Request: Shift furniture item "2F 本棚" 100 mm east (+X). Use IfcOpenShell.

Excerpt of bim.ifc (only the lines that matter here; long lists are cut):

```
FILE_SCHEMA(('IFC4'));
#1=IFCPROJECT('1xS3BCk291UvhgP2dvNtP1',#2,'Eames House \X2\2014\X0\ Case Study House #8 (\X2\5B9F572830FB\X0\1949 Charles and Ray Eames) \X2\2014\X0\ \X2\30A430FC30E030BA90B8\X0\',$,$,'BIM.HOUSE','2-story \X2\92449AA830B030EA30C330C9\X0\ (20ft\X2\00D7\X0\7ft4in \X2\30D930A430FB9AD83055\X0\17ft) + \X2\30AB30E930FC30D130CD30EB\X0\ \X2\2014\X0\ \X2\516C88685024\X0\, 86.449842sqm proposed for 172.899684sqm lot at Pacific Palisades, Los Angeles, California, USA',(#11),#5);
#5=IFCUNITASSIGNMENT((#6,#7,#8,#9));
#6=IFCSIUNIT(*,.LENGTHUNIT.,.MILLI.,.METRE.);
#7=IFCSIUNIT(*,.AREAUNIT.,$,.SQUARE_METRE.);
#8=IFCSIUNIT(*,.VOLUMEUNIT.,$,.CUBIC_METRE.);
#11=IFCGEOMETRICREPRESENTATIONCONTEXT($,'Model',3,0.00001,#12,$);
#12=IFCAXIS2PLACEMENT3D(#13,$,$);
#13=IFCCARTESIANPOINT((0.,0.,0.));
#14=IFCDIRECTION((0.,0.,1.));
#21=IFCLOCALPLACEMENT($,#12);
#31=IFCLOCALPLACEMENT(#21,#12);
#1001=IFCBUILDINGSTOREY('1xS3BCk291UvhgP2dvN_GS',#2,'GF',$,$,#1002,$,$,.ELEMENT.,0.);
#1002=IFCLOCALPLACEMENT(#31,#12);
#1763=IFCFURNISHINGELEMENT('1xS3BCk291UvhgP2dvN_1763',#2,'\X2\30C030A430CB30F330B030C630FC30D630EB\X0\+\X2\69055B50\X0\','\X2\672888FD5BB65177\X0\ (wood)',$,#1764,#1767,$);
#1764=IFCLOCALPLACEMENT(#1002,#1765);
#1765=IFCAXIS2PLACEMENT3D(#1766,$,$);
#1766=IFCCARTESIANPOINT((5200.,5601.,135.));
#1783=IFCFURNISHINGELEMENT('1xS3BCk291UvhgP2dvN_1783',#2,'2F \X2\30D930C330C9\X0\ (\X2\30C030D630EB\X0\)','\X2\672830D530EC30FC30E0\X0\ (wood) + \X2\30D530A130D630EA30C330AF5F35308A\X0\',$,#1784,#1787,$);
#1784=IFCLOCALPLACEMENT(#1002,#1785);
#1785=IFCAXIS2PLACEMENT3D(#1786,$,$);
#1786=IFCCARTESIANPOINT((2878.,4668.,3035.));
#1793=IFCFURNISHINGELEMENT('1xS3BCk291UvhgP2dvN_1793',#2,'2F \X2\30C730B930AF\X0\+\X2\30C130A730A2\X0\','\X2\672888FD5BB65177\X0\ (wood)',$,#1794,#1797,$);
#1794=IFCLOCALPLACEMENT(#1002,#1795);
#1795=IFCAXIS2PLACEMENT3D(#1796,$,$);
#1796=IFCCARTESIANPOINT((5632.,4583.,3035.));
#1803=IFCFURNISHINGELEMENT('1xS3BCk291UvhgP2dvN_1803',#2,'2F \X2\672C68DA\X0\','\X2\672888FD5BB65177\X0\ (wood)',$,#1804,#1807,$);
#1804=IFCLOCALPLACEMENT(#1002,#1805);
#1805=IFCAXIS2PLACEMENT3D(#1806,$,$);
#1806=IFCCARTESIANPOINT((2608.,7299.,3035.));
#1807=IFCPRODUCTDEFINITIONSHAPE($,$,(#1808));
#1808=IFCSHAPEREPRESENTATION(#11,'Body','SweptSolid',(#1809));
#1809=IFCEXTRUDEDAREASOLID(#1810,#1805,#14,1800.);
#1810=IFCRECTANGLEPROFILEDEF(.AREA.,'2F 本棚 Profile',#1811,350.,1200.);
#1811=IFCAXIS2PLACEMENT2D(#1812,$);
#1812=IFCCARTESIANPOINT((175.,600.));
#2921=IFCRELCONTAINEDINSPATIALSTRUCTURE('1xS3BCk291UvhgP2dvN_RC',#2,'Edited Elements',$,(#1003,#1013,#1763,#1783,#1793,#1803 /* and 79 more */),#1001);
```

```python
import ifcopenshell
import ifcopenshell.api.geometry
import ifcopenshell.util.placement
import ifcopenshell.util.unit

model = ifcopenshell.open("bim.ifc")
unit_scale = ifcopenshell.util.unit.calculate_unit_scale(model)

item = model.by_guid("1xS3BCk291UvhgP2dvN_1803")
matrix = ifcopenshell.util.placement.get_local_placement(item.ObjectPlacement)
matrix[0, 3] += 0.1 / unit_scale
ifcopenshell.api.geometry.edit_object_placement(model, product=item, matrix=matrix, is_si=False)

print(ifcopenshell.util.placement.get_local_placement(item.ObjectPlacement).round(3) + 0.0)

model.write("bim_v2.ifc")
```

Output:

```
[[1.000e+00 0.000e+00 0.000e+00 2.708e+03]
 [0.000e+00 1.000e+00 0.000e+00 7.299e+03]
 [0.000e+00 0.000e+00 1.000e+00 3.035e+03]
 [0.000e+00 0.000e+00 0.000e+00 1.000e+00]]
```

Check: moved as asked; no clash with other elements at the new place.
